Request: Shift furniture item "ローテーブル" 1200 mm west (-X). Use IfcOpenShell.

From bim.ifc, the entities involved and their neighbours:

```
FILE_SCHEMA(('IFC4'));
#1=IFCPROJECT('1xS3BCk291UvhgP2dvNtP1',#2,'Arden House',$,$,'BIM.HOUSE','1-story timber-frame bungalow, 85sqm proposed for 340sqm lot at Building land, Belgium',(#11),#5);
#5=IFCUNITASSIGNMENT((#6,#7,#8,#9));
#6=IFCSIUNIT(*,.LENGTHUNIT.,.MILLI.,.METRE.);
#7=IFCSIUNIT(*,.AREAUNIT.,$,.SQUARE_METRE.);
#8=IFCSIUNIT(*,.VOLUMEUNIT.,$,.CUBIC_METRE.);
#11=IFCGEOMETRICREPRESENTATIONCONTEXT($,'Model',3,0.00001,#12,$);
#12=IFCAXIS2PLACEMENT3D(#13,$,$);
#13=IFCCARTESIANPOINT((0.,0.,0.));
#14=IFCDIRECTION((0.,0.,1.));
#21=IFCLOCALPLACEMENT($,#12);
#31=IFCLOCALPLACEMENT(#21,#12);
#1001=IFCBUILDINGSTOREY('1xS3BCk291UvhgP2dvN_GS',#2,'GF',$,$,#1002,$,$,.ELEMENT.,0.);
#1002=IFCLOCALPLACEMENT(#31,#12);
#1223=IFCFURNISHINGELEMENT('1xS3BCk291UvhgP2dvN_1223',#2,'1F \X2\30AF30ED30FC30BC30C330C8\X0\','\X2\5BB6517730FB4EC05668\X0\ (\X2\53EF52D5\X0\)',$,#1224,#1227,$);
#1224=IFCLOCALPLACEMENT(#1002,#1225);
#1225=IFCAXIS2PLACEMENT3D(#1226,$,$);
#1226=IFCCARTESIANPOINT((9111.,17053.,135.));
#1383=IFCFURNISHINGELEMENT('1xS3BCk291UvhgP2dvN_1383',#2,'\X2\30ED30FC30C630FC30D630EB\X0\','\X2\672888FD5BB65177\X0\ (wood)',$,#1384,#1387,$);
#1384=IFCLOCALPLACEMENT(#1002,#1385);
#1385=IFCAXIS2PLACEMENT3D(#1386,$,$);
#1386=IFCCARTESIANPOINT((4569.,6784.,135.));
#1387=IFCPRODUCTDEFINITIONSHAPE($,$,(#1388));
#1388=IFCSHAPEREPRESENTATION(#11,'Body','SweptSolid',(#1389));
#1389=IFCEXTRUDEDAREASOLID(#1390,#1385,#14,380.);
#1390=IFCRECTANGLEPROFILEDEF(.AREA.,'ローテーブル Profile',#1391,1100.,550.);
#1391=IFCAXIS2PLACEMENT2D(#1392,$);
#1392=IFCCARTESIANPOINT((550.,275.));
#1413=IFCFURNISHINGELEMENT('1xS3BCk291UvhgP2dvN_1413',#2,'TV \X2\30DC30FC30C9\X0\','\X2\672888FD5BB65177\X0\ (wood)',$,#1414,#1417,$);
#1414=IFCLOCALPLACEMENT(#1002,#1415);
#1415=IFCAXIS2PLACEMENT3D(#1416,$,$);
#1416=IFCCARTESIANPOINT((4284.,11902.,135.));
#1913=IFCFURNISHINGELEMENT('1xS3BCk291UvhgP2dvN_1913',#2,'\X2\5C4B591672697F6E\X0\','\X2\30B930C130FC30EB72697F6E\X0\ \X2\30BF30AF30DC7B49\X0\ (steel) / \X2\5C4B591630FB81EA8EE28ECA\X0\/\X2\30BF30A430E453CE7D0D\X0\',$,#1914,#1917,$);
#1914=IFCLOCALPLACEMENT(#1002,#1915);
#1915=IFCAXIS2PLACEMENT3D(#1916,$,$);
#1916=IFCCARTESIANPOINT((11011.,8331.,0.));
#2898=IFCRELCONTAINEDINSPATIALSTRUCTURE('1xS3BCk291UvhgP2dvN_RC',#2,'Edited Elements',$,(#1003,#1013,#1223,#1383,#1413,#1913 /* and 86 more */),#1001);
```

```python
import ifcopenshell
import ifcopenshell.api.geometry
import ifcopenshell.util.placement

model = ifcopenshell.open("bim.ifc")

item = model.by_guid("1xS3BCk291UvhgP2dvN_1383")
matrix = ifcopenshell.util.placement.get_local_placement(item.ObjectPlacement)
matrix[0, 3] -= 1200.0
ifcopenshell.api.geometry.edit_object_placement(model, product=item, matrix=matrix, is_si=False)

print(ifcopenshell.util.placement.get_local_placement(item.ObjectPlacement).round(3) + 0.0)

model.write("bim_v2.ifc")
```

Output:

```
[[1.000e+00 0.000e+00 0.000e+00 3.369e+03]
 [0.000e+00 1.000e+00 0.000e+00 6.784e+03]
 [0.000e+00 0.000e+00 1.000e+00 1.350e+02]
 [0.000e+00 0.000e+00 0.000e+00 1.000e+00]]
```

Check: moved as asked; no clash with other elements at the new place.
